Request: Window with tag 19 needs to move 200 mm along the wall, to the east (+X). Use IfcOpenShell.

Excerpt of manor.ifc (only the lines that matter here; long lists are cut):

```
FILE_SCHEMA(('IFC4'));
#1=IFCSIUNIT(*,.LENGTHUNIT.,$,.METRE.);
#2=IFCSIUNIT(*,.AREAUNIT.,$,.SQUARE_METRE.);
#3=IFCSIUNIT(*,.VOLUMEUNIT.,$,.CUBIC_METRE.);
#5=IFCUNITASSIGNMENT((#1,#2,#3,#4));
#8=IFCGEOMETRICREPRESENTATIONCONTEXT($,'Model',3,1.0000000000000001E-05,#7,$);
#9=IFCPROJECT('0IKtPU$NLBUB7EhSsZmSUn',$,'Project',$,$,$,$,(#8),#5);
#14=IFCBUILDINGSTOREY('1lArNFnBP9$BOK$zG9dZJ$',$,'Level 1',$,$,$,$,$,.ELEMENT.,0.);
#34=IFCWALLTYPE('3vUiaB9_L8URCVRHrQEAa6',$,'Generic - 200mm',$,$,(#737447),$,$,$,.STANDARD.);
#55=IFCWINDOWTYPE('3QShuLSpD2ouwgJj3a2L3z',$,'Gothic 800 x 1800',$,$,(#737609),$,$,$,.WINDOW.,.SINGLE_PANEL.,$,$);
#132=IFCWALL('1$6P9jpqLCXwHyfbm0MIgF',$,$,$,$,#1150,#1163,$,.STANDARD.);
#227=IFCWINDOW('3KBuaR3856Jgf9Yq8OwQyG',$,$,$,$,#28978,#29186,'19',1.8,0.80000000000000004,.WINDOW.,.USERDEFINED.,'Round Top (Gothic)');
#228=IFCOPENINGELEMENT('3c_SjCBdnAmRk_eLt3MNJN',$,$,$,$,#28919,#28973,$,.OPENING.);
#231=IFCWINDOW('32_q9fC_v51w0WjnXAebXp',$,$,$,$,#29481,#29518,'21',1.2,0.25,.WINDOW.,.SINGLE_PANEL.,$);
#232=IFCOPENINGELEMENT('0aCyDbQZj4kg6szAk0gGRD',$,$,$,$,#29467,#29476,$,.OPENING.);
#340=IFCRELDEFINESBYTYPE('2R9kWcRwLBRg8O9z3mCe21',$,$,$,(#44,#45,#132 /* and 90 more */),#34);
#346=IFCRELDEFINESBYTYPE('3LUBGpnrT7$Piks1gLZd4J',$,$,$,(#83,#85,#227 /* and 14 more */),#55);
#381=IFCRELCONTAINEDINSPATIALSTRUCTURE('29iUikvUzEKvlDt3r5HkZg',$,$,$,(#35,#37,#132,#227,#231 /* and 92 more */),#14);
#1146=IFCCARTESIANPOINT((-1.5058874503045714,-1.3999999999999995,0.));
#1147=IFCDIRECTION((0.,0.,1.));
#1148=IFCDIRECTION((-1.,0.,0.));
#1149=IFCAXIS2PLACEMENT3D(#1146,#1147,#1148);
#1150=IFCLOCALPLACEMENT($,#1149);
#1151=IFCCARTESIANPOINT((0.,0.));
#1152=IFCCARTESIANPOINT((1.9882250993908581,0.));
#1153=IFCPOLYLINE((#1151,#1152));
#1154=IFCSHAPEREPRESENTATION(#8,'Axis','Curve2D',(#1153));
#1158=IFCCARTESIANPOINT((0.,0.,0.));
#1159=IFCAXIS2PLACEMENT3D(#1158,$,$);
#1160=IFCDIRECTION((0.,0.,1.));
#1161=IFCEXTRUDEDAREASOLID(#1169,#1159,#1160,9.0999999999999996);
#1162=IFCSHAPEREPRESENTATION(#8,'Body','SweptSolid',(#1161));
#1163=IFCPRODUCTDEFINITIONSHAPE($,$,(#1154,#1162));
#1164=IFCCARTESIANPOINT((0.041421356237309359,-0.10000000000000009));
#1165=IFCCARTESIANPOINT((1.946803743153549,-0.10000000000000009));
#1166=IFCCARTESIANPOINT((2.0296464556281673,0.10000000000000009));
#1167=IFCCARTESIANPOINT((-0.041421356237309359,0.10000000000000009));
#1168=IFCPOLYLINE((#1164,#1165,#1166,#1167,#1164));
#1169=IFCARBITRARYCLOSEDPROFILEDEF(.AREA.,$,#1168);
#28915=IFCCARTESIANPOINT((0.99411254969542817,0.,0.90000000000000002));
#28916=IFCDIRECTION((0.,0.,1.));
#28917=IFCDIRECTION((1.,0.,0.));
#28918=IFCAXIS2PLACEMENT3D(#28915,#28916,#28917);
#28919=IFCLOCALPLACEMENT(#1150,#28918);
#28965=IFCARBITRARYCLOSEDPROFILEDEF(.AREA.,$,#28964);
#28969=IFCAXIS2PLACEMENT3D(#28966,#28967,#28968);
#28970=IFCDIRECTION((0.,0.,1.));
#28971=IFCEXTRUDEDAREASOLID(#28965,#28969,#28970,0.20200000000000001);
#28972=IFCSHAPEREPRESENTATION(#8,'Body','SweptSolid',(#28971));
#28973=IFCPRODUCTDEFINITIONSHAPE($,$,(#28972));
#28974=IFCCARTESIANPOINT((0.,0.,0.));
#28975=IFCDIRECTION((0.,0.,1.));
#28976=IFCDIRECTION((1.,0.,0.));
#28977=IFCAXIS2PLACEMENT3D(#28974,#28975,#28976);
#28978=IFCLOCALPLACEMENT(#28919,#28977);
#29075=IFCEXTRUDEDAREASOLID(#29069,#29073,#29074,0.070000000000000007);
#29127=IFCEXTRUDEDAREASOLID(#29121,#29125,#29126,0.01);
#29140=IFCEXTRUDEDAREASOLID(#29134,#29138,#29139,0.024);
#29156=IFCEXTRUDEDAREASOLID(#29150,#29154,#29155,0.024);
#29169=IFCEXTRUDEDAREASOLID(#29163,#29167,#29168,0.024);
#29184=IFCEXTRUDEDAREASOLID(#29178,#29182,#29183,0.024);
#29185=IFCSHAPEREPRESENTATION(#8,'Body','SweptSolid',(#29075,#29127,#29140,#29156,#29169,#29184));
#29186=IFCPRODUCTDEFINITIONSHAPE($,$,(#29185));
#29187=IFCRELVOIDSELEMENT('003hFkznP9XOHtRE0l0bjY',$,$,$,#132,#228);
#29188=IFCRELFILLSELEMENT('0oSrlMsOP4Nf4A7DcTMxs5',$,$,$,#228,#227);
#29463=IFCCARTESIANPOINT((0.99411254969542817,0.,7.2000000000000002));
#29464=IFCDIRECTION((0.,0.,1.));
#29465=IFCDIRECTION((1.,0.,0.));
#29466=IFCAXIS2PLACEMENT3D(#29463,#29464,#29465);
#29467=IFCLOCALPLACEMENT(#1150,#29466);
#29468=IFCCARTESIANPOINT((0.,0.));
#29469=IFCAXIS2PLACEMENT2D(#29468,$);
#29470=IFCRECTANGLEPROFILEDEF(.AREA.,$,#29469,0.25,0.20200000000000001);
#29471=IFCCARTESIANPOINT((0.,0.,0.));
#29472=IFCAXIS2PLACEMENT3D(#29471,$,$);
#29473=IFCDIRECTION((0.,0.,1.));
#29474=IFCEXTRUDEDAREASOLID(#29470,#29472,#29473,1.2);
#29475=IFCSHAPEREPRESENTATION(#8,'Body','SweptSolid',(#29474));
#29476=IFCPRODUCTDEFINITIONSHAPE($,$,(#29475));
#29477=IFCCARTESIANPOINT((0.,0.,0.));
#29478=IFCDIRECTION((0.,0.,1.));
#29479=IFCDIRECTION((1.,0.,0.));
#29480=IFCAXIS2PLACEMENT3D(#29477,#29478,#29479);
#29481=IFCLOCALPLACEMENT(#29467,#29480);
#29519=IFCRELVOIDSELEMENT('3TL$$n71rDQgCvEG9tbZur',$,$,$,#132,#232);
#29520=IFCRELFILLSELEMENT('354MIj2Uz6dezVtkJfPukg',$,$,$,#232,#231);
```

```python
import ifcopenshell
import ifcopenshell.api.geometry
import ifcopenshell.util.placement

model = ifcopenshell.open("manor.ifc")

window = model.by_id(227)
opening = window.FillsVoids[0].RelatingOpeningElement
wall = opening.VoidsElements[0].RelatingBuildingElement

wall_matrix = ifcopenshell.util.placement.get_local_placement(wall.ObjectPlacement)
shift = wall_matrix[:3, 0] * -0.2
before = ifcopenshell.util.placement.get_local_placement(window.ObjectPlacement)[:3, 3].copy()

# The window is placed relative to its opening, so it follows when the opening moves.
matrix = ifcopenshell.util.placement.get_local_placement(opening.ObjectPlacement)
matrix[:3, 3] += shift
ifcopenshell.api.geometry.edit_object_placement(
    model, product=opening, matrix=matrix, is_si=False, should_transform_children=True
)

after = ifcopenshell.util.placement.get_local_placement(window.ObjectPlacement)[:3, 3]
print("window moved by", (after - before).round(3) + 0.0)

model.write("manor_rev.ifc")
```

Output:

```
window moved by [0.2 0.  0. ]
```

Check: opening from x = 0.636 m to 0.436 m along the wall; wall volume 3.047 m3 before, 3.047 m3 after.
